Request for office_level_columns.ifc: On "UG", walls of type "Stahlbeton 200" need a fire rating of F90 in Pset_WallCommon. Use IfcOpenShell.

First a look at what the model holds.

```python
import ifcopenshell
import ifcopenshell.util.element

model = ifcopenshell.open("office_level_columns.ifc")
print(model.schema)
storey = next(s for s in model.by_type("IfcBuildingStorey") if s.Name == "UG")
walls = [e for e in ifcopenshell.util.element.get_decomposition(storey) if e.is_a("IfcWall")]
seen = {}
for e in walls:
    element_type = ifcopenshell.util.element.get_type(e)
    key = (element_type.Name if element_type != e and element_type else None, ifcopenshell.util.element.get_pset(e, "Pset_WallCommon", "FireRating"))
    seen[key] = seen.get(key, 0) + 1
for (name, value), count in sorted(seen.items(), key=str):
    print(count, "x", name, "|", value)
```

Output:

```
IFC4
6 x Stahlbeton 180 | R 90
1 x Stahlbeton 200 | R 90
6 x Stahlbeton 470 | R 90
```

```python
import ifcopenshell
import ifcopenshell.api.pset
import ifcopenshell.util.element

model = ifcopenshell.open("office_level_columns.ifc")

storey = next(s for s in model.by_type("IfcBuildingStorey") if s.Name == "UG")
walls = [e for e in ifcopenshell.util.element.get_decomposition(storey) if e.is_a("IfcWall")]

count = 0
for e in walls:
    element_type = ifcopenshell.util.element.get_type(e)
    if element_type in (None, e) or element_type.Name != "Stahlbeton 200":
        continue
    # add_pset returns the element's existing set when there is one.
    pset = ifcopenshell.api.pset.add_pset(model, product=e, name="Pset_WallCommon")
    ifcopenshell.api.pset.edit_pset(model, pset=pset, properties={"FireRating": "F90"})
    count += 1

print(count, "walls updated")

model.write("office_level_columns-out.ifc")
```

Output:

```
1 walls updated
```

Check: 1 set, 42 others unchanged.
